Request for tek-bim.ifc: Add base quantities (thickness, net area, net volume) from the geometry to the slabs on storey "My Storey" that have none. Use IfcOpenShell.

First a look at what the model holds.

```python
import ifcopenshell
import ifcopenshell.util.element
import ifcopenshell.util.unit

model = ifcopenshell.open("tek-bim.ifc")
print(model.schema)
for unit_type in ("LENGTHUNIT", "AREAUNIT", "VOLUMEUNIT"):
    print(unit_type, ifcopenshell.util.unit.calculate_unit_scale(model, unit_type))
storey = next(s for s in model.by_type("IfcBuildingStorey") if s.Name == "My Storey")
slabs = [e for e in ifcopenshell.util.element.get_decomposition(storey) if e.is_a("IfcSlab")]
for e in sorted(slabs, key=lambda e: e.id()):
    print(e.id(), e.is_a(), e.Name, list(ifcopenshell.util.element.get_psets(e, qtos_only=True)), sep=" | ")
```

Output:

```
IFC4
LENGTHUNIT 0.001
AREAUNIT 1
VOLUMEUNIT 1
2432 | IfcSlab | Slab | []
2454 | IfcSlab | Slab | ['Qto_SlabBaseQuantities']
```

```python
import ifcopenshell
import ifcopenshell.api.pset
import ifcopenshell.geom
import ifcopenshell.util.element
import ifcopenshell.util.shape
import ifcopenshell.util.unit

model = ifcopenshell.open("tek-bim.ifc")
unit_scale = ifcopenshell.util.unit.calculate_unit_scale(model)
area_scale = ifcopenshell.util.unit.calculate_unit_scale(model, "AREAUNIT")
volume_scale = ifcopenshell.util.unit.calculate_unit_scale(model, "VOLUMEUNIT")
settings = ifcopenshell.geom.settings()

storey = next(s for s in model.by_type("IfcBuildingStorey") if s.Name == "My Storey")
slabs = [e for e in ifcopenshell.util.element.get_decomposition(storey) if e.is_a("IfcSlab")]

for e in sorted(slabs, key=lambda e: e.id()):
    if ifcopenshell.util.element.get_psets(e, qtos_only=True, should_inherit=False):
        continue
    # Geometry comes back in metres, in the element's own axes.
    shape = ifcopenshell.geom.create_shape(settings, e)
    values = {
        "Width": ifcopenshell.util.shape.get_z(shape.geometry) / unit_scale,
        "NetArea": ifcopenshell.util.shape.get_footprint_area(shape.geometry) / area_scale,
        "NetVolume": ifcopenshell.util.shape.get_volume(shape.geometry) / volume_scale,
    }
    qto = ifcopenshell.api.pset.add_qto(model, product=e, name="Qto_SlabBaseQuantities")
    ifcopenshell.api.pset.edit_qto(model, qto=qto, properties=values)
    print(e.id(), {k: round(v, 3) for k, v in values.items()})

model.write("tek-bim_edited.ifc")
```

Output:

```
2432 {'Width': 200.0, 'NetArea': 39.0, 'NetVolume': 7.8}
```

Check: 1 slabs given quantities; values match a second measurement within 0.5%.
